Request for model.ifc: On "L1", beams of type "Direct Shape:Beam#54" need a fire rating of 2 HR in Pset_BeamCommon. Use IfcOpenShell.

First a look at what the model holds.

```python
import ifcopenshell
import ifcopenshell.util.element

model = ifcopenshell.open("model.ifc")
print(model.schema)
storey = next(s for s in model.by_type("IfcBuildingStorey") if s.Name == "L1")
beams = [e for e in ifcopenshell.util.element.get_decomposition(storey) if e.is_a("IfcBeam")]
seen = {}
for e in beams:
    element_type = ifcopenshell.util.element.get_type(e)
    key = (element_type.Name if element_type != e and element_type else None, ifcopenshell.util.element.get_pset(e, "Pset_BeamCommon", "FireRating"))
    seen[key] = seen.get(key, 0) + 1
for (name, value), count in sorted(seen.items(), key=str):
    print(count, "x", name, "|", value)
```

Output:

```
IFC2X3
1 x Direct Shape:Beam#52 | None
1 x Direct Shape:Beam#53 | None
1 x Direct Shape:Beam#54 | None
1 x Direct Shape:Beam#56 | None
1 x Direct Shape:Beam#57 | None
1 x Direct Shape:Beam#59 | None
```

```python
import ifcopenshell
import ifcopenshell.api.pset
import ifcopenshell.util.element

model = ifcopenshell.open("model.ifc")

storey = next(s for s in model.by_type("IfcBuildingStorey") if s.Name == "L1")
beams = [e for e in ifcopenshell.util.element.get_decomposition(storey) if e.is_a("IfcBeam")]

count = 0
for e in beams:
    element_type = ifcopenshell.util.element.get_type(e)
    if element_type in (None, e) or element_type.Name != "Direct Shape:Beam#54":
        continue
    # add_pset returns the element's existing set when there is one.
    pset = ifcopenshell.api.pset.add_pset(model, product=e, name="Pset_BeamCommon")
    ifcopenshell.api.pset.edit_pset(model, pset=pset, properties={"FireRating": "2 HR"})
    count += 1

print(count, "beams updated")

model.write("model_edited.ifc")
```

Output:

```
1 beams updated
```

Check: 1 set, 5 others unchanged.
